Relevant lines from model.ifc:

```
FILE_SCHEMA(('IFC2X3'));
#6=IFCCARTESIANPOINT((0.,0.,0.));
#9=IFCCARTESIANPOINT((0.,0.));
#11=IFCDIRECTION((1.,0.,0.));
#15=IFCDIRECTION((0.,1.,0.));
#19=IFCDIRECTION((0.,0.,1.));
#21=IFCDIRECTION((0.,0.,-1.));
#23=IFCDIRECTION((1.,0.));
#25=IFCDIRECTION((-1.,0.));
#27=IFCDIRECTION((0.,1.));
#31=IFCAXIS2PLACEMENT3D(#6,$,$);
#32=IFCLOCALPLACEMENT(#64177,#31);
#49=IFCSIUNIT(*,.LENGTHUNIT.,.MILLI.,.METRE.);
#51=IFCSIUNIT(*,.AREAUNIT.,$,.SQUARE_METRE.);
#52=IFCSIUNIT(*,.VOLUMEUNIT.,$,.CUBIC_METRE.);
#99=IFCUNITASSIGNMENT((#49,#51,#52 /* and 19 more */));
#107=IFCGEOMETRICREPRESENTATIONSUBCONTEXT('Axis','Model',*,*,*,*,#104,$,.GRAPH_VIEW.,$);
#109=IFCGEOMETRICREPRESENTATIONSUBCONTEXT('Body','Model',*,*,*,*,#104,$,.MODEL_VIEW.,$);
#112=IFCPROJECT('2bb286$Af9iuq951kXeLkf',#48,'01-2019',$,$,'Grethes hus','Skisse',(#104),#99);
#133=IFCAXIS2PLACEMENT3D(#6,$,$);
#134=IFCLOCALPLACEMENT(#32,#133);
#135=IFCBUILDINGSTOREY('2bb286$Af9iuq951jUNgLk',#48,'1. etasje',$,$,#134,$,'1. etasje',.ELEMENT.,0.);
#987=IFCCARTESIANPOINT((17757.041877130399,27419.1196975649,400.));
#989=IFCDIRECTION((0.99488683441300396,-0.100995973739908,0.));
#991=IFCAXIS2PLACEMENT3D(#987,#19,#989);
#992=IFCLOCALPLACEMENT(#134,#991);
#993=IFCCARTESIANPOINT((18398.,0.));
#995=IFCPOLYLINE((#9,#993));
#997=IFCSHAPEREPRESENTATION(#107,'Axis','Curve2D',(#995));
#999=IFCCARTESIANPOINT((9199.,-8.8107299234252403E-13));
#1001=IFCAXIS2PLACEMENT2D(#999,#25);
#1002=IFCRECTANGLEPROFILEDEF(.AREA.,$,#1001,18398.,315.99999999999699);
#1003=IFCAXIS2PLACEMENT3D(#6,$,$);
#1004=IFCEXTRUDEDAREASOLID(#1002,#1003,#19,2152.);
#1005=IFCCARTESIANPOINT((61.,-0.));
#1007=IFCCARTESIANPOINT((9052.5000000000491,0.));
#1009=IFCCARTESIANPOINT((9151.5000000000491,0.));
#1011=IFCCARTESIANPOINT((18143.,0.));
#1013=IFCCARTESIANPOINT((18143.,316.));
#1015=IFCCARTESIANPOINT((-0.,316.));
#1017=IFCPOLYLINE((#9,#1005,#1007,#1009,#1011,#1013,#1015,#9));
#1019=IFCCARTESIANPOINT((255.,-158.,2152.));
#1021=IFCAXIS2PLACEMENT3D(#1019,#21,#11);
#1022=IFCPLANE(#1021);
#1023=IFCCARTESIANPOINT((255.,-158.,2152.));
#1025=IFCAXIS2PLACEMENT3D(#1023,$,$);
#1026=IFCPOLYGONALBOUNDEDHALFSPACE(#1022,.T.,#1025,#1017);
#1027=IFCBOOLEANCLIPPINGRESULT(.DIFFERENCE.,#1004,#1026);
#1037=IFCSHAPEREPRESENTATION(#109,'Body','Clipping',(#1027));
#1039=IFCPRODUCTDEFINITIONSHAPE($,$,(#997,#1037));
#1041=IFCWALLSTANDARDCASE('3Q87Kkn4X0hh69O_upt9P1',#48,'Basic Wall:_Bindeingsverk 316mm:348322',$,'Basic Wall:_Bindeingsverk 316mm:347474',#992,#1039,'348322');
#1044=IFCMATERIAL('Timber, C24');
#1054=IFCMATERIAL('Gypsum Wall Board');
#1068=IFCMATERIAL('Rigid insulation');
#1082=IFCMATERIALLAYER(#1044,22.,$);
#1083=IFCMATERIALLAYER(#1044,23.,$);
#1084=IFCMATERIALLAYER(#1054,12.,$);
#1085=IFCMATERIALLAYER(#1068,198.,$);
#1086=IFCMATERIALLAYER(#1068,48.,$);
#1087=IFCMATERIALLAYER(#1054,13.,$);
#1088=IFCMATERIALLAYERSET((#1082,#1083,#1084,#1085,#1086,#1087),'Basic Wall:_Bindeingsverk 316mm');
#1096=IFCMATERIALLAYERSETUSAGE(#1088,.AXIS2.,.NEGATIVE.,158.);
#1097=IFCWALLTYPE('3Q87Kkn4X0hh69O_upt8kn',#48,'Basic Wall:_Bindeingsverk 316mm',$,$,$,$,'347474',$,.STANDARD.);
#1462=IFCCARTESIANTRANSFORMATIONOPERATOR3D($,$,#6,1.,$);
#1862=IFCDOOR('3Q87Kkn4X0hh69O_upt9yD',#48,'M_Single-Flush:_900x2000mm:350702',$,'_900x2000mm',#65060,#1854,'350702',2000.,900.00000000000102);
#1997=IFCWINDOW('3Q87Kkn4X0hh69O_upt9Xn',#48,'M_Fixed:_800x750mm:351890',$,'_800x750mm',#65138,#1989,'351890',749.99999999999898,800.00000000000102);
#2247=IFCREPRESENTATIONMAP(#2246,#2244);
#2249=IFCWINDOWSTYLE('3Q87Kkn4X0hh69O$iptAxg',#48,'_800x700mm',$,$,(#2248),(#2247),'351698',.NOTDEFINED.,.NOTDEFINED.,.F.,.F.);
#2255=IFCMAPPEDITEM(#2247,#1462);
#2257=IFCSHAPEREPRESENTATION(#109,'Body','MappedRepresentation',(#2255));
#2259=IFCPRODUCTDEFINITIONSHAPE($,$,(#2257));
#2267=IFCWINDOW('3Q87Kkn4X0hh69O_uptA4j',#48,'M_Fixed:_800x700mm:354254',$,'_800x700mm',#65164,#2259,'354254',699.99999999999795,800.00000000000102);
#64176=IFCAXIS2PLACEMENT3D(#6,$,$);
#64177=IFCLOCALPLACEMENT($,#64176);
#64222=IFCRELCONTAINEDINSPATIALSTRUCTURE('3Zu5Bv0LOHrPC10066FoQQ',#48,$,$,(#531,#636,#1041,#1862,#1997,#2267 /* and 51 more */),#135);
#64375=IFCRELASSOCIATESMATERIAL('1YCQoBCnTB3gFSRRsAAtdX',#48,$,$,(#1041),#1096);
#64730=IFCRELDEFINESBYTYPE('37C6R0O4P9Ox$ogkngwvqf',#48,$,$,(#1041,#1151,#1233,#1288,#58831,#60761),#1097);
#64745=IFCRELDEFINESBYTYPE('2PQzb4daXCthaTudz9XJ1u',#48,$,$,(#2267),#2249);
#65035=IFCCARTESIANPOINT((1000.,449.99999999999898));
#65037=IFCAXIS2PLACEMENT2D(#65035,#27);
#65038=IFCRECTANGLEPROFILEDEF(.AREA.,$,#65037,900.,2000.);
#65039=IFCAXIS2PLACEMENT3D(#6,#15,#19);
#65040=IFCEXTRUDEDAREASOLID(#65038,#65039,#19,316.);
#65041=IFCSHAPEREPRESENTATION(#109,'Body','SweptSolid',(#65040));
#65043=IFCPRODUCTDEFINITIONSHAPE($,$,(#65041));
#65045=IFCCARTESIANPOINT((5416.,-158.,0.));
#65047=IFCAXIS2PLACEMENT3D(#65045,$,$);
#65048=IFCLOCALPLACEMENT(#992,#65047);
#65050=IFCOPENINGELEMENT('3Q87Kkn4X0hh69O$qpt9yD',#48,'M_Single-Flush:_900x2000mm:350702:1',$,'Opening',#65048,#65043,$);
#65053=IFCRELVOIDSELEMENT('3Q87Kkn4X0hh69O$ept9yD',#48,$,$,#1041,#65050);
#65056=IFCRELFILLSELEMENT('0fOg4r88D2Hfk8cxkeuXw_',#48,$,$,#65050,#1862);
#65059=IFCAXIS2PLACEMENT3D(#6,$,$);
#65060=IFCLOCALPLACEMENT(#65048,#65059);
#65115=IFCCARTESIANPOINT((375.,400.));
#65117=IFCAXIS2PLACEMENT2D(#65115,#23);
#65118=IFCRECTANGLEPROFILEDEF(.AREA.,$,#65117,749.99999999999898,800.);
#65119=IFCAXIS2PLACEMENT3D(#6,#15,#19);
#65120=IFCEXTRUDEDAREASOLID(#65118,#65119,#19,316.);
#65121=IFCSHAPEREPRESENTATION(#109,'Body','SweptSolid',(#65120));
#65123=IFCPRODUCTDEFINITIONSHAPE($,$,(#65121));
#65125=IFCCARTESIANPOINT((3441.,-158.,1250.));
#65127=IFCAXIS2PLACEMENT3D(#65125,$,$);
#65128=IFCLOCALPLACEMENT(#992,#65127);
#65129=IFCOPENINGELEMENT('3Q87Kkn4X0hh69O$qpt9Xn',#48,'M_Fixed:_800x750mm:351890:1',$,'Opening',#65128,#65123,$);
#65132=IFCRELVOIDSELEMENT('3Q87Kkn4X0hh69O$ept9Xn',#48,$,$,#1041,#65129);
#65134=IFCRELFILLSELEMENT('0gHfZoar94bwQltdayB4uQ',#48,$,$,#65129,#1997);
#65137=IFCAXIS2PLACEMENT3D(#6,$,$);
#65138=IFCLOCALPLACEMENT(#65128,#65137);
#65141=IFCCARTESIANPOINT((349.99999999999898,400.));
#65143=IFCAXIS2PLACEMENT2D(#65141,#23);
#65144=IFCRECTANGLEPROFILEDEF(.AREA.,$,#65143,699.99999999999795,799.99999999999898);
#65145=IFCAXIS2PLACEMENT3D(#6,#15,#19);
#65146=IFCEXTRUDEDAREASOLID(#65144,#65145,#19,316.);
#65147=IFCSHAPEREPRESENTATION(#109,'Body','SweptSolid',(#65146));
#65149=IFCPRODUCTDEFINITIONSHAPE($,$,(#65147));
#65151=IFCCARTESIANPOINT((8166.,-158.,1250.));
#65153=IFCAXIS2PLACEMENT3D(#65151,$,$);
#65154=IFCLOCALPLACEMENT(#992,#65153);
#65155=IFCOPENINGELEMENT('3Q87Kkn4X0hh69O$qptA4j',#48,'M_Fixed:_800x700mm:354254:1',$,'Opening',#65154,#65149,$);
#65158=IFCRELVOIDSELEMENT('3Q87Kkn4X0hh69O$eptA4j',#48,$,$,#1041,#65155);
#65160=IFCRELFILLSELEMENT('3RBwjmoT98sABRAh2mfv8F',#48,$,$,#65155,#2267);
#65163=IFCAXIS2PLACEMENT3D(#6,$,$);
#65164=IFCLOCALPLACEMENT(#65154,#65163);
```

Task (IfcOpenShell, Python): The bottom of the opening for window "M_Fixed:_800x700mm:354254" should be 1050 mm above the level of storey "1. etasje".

```python
import numpy as np
import ifcopenshell
import ifcopenshell.api.geometry
import ifcopenshell.geom
import ifcopenshell.util.element
import ifcopenshell.util.placement
import ifcopenshell.util.shape
import ifcopenshell.util.unit

model = ifcopenshell.open("model.ifc")
unit_scale = ifcopenshell.util.unit.calculate_unit_scale(model)

window = model.by_id(2267)
opening = window.FillsVoids[0].RelatingOpeningElement
storey = ifcopenshell.util.element.get_container(window, ifc_class="IfcBuildingStorey")
level = ifcopenshell.util.placement.get_local_placement(storey.ObjectPlacement)[2, 3]

# The opening's origin need not be at the sill, so measure its lowest point.
shape = ifcopenshell.geom.create_shape(ifcopenshell.geom.settings(), opening)
bottom = ifcopenshell.util.shape.get_shape_bottom_elevation(shape, shape.geometry) / unit_scale
dz = level + 1.05 / unit_scale - bottom

shift = np.array([0.0, 0.0, dz])
# The window is placed relative to its opening, so it follows when the opening moves.
matrix = ifcopenshell.util.placement.get_local_placement(opening.ObjectPlacement)
matrix[:3, 3] += shift
ifcopenshell.api.geometry.edit_object_placement(
    model, product=opening, matrix=matrix, is_si=False, should_transform_children=True
)

print(f"moved by {dz * unit_scale:+.3f} m")

model.write("model_rev.ifc")
```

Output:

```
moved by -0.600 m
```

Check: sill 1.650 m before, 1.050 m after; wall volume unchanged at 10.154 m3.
